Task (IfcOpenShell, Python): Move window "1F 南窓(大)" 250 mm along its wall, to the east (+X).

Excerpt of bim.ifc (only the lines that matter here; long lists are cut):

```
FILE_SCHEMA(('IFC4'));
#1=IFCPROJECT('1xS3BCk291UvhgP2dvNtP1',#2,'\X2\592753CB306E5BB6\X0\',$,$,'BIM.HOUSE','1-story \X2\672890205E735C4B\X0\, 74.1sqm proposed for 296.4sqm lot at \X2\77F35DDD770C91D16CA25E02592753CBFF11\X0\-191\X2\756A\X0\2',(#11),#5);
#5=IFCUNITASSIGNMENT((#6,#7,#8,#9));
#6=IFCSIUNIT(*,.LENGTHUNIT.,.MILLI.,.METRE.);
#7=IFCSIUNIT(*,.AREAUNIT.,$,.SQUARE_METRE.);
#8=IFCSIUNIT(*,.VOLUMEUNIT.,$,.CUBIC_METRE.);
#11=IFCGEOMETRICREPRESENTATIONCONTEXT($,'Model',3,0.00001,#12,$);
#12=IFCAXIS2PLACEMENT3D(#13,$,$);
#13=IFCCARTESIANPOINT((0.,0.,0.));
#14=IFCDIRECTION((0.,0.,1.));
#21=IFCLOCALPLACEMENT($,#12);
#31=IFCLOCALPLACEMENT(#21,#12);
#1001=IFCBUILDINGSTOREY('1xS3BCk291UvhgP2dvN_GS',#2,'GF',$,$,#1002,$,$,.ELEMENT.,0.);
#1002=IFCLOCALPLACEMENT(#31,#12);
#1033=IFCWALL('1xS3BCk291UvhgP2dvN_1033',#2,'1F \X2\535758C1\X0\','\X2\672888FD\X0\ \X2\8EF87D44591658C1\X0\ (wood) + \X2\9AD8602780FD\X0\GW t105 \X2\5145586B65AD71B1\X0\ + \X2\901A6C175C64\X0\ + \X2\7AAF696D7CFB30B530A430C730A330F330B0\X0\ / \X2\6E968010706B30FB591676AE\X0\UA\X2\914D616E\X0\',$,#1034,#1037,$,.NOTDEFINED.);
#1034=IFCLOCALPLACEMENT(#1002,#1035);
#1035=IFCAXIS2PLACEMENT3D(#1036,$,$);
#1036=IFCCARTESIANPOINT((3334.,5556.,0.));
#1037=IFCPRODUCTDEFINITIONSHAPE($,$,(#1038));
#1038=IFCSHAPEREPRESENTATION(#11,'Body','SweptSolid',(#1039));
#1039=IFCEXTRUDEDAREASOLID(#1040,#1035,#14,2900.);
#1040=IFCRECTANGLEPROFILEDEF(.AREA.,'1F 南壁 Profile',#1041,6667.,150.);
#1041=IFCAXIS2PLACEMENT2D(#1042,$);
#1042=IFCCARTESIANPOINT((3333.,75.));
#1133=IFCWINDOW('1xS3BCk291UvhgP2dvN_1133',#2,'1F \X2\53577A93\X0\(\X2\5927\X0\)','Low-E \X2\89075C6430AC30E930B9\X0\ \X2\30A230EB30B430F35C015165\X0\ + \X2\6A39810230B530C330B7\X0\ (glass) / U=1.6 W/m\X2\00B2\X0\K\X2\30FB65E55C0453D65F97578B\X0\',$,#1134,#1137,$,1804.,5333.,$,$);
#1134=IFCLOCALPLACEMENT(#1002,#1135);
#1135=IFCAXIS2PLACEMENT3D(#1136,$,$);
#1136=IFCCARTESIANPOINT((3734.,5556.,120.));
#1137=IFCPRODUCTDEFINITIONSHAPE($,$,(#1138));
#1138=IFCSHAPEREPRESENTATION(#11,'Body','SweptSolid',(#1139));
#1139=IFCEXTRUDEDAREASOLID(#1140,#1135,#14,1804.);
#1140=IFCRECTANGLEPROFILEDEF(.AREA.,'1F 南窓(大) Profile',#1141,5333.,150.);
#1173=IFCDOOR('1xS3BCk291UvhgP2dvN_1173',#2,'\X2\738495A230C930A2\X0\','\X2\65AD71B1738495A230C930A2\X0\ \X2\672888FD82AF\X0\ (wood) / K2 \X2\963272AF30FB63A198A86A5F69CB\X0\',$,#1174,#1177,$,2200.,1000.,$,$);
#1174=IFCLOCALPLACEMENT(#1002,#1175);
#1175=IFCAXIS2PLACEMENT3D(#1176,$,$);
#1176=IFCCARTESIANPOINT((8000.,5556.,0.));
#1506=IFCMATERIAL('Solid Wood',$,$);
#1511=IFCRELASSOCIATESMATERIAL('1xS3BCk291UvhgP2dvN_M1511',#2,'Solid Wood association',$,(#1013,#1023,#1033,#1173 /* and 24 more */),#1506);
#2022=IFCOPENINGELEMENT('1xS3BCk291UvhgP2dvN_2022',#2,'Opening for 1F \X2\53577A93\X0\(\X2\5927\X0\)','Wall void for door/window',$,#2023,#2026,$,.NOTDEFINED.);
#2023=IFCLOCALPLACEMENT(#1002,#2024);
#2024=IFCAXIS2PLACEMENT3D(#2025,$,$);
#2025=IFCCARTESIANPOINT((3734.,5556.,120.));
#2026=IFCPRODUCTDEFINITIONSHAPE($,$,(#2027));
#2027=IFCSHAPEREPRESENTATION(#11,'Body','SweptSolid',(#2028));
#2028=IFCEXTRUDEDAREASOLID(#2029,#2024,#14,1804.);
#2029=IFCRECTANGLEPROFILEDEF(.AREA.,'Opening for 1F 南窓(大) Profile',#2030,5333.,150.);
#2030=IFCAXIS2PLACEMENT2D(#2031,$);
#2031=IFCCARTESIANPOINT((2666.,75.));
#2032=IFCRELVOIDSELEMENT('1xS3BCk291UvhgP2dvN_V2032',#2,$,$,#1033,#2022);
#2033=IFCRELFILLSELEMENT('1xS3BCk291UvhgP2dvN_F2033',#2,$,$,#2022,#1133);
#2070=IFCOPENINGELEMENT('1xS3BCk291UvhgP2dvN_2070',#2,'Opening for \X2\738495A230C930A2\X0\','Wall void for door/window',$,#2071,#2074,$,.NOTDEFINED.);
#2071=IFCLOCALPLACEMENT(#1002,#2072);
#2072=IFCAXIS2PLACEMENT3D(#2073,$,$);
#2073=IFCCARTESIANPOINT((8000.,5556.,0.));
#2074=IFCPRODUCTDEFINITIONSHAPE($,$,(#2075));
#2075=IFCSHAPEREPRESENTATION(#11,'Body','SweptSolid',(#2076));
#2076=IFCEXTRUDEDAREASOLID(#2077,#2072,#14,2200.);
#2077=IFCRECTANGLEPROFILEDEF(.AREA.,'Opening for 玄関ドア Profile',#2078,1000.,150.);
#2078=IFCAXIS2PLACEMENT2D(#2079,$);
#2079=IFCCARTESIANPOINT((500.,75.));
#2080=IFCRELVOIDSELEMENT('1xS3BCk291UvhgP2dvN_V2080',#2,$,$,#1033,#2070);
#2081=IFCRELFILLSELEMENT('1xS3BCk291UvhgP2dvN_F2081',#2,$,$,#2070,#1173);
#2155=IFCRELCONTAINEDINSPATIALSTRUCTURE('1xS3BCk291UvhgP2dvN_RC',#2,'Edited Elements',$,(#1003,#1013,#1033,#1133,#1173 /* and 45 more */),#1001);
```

```python
import ifcopenshell
import ifcopenshell.api.geometry
import ifcopenshell.util.placement
import ifcopenshell.util.unit

model = ifcopenshell.open("bim.ifc")
unit_scale = ifcopenshell.util.unit.calculate_unit_scale(model)

window = model.by_guid("1xS3BCk291UvhgP2dvN_1133")
opening = window.FillsVoids[0].RelatingOpeningElement
wall = opening.VoidsElements[0].RelatingBuildingElement

wall_matrix = ifcopenshell.util.placement.get_local_placement(wall.ObjectPlacement)
shift = wall_matrix[:3, 0] * 0.25 / unit_scale
before = ifcopenshell.util.placement.get_local_placement(window.ObjectPlacement)[:3, 3].copy()

# The window is not placed relative to its opening, so move both.
for product in (opening, window):
    matrix = ifcopenshell.util.placement.get_local_placement(product.ObjectPlacement)
    matrix[:3, 3] += shift
    ifcopenshell.api.geometry.edit_object_placement(model, product=product, matrix=matrix, is_si=False)

after = ifcopenshell.util.placement.get_local_placement(window.ObjectPlacement)[:3, 3]
print("window moved by", (after - before).round(3) + 0.0)

model.write("bim_v2.ifc")
```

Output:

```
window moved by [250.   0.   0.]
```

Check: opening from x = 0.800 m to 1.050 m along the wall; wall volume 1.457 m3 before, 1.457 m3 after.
